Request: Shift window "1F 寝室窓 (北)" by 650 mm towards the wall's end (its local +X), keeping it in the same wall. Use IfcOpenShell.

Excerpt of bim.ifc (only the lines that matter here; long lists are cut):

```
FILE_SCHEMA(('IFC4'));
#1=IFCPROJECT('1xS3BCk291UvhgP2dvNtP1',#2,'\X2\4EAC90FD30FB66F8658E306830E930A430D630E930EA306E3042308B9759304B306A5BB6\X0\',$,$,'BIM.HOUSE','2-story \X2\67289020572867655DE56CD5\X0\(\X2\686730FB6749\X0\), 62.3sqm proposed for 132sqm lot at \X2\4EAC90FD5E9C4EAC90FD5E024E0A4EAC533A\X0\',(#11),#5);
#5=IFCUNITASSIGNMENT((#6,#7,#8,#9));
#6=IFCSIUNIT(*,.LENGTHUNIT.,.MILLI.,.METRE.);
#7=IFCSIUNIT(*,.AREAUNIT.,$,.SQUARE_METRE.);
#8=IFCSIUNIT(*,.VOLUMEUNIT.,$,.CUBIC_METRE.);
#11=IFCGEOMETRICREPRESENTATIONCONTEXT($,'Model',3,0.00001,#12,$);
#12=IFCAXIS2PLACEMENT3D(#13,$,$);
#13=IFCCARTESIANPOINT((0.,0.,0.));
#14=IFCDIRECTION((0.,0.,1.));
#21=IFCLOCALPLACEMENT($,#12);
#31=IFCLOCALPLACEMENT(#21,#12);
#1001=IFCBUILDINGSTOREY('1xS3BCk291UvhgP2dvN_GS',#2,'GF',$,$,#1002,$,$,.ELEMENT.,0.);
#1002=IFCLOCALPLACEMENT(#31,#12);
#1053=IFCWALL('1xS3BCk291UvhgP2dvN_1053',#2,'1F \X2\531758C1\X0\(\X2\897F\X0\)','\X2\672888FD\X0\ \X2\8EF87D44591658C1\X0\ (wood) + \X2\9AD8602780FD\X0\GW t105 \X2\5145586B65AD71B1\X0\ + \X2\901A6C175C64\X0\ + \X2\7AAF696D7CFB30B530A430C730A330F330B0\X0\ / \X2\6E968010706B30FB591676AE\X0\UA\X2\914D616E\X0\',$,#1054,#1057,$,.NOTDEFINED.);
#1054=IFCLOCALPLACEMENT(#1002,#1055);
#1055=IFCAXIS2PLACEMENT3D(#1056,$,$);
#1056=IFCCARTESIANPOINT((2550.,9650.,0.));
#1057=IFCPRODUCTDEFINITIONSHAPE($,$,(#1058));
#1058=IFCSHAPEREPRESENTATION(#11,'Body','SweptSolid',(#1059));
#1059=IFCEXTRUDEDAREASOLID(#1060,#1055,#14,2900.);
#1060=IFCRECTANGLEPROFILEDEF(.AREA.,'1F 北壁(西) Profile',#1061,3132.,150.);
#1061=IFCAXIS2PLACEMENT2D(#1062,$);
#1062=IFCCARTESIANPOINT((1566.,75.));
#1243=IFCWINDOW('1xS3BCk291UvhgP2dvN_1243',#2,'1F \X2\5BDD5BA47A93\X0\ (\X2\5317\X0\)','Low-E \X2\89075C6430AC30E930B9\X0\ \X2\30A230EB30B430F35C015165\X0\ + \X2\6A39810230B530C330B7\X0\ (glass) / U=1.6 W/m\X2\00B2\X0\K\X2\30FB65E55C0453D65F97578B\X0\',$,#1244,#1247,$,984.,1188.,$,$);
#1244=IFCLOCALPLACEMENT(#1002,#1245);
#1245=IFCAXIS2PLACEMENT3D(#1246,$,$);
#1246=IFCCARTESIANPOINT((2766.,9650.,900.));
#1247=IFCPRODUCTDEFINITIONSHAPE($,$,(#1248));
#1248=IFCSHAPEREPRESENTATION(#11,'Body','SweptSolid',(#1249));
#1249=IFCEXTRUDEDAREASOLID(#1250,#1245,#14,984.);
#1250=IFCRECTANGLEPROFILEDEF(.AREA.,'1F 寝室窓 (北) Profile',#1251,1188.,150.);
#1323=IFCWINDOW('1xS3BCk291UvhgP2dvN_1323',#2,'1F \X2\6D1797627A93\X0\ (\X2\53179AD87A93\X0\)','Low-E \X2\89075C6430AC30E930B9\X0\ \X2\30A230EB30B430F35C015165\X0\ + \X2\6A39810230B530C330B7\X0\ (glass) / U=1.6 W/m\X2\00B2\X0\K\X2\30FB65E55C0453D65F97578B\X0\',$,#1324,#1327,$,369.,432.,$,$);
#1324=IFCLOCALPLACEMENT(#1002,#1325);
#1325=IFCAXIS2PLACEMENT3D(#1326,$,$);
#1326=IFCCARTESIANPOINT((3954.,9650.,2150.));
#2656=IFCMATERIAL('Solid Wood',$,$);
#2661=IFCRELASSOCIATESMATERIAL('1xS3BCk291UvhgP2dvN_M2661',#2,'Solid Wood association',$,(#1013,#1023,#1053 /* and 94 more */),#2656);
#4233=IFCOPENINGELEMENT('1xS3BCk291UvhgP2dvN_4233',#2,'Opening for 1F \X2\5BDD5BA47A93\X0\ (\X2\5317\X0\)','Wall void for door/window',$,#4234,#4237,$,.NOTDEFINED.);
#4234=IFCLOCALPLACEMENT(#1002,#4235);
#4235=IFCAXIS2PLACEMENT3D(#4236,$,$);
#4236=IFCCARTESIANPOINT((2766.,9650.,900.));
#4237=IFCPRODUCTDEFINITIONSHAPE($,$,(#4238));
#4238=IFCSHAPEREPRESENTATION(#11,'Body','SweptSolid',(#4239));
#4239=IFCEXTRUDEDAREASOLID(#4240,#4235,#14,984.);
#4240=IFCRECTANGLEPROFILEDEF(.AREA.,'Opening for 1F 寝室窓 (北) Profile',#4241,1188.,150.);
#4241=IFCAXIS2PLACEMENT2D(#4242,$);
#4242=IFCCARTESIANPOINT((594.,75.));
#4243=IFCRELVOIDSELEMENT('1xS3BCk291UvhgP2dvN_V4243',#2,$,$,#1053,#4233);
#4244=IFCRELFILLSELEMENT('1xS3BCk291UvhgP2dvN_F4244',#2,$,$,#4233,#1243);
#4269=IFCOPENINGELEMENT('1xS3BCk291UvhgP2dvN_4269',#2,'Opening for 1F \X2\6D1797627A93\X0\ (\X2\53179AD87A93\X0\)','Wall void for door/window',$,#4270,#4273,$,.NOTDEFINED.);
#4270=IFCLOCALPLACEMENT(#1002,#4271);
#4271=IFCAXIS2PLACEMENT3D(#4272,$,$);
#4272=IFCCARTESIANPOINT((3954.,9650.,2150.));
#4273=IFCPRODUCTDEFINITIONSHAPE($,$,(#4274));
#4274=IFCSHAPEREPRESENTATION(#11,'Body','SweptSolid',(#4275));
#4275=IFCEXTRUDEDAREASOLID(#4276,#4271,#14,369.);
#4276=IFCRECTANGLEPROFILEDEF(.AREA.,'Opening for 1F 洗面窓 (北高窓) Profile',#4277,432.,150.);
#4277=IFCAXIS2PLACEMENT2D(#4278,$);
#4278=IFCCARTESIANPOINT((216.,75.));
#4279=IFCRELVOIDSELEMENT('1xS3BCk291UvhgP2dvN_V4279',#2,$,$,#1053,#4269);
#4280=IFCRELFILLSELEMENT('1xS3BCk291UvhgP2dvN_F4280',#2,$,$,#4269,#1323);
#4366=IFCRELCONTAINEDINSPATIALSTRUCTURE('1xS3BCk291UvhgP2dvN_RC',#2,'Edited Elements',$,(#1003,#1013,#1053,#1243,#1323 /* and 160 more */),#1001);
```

```python
import ifcopenshell
import ifcopenshell.api.geometry
import ifcopenshell.util.placement

model = ifcopenshell.open("bim.ifc")

window = model.by_id(1243)
opening = window.FillsVoids[0].RelatingOpeningElement
wall = opening.VoidsElements[0].RelatingBuildingElement

wall_matrix = ifcopenshell.util.placement.get_local_placement(wall.ObjectPlacement)
shift = wall_matrix[:3, 0] * 650.0
before = ifcopenshell.util.placement.get_local_placement(window.ObjectPlacement)[:3, 3].copy()

# The window is not placed relative to its opening, so move both.
for product in (opening, window):
    matrix = ifcopenshell.util.placement.get_local_placement(product.ObjectPlacement)
    matrix[:3, 3] += shift
    ifcopenshell.api.geometry.edit_object_placement(model, product=product, matrix=matrix, is_si=False)

after = ifcopenshell.util.placement.get_local_placement(window.ObjectPlacement)[:3, 3]
print("window moved by", (after - before).round(3) + 0.0)

model.write("bim-out.ifc")
```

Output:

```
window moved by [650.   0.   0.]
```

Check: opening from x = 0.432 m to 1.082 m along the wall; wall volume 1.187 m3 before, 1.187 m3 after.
